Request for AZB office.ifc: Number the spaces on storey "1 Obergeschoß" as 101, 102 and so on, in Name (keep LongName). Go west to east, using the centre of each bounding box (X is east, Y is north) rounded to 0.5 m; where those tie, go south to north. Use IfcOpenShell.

First a look at what the model holds.

```python
import ifcopenshell
import ifcopenshell.util.element
import ifcopenshell.util.placement

model = ifcopenshell.open("AZB office.ifc")
print(model.schema)
storey = next(s for s in model.by_type("IfcBuildingStorey") if s.Name == "1 Obergeschoß")
spaces = [e for e in ifcopenshell.util.element.get_decomposition(storey) if e.is_a("IfcSpace")]
for e in sorted(spaces, key=lambda e: e.id()):
    origin = ifcopenshell.util.placement.get_local_placement(e.ObjectPlacement)[:3, 3]
    print(e.id(), e.Name, e.LongName, origin.round(2) + 0.0, sep=" | ")
```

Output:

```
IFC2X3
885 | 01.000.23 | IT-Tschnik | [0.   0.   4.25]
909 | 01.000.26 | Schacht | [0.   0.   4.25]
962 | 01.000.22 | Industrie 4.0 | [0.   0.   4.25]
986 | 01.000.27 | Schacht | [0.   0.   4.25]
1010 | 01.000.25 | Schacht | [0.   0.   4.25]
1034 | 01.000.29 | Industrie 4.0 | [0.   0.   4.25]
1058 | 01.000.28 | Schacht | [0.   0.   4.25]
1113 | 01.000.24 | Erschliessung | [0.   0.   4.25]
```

```python
import ifcopenshell
import ifcopenshell.geom
import ifcopenshell.util.element
import ifcopenshell.util.shape

model = ifcopenshell.open("AZB office.ifc")
settings = ifcopenshell.geom.settings()
settings.set("use-world-coords", True)


def centre(element):
    shape = ifcopenshell.geom.create_shape(settings, element)
    return ifcopenshell.util.shape.get_bbox_centroid(shape.geometry)


storey = next(s for s in model.by_type("IfcBuildingStorey") if s.Name == "1 Obergeschoß")
spaces = [e for e in ifcopenshell.util.element.get_decomposition(storey) if e.is_a("IfcSpace")]

# Insertion points can sit at a corner or the storey origin, so sort by the geometry (in metres).
centres = {e: centre(e) for e in spaces}
spaces.sort(key=lambda e: (round(centres[e][0] / 0.5), centres[e][1]))

for i, e in enumerate(spaces, start=1):
    number = f"1{i:02d}"
    e.Name = number
    print(e.id(), number)

model.write("AZB office_updated.ifc")
```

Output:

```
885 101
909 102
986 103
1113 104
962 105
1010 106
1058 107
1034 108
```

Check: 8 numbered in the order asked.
